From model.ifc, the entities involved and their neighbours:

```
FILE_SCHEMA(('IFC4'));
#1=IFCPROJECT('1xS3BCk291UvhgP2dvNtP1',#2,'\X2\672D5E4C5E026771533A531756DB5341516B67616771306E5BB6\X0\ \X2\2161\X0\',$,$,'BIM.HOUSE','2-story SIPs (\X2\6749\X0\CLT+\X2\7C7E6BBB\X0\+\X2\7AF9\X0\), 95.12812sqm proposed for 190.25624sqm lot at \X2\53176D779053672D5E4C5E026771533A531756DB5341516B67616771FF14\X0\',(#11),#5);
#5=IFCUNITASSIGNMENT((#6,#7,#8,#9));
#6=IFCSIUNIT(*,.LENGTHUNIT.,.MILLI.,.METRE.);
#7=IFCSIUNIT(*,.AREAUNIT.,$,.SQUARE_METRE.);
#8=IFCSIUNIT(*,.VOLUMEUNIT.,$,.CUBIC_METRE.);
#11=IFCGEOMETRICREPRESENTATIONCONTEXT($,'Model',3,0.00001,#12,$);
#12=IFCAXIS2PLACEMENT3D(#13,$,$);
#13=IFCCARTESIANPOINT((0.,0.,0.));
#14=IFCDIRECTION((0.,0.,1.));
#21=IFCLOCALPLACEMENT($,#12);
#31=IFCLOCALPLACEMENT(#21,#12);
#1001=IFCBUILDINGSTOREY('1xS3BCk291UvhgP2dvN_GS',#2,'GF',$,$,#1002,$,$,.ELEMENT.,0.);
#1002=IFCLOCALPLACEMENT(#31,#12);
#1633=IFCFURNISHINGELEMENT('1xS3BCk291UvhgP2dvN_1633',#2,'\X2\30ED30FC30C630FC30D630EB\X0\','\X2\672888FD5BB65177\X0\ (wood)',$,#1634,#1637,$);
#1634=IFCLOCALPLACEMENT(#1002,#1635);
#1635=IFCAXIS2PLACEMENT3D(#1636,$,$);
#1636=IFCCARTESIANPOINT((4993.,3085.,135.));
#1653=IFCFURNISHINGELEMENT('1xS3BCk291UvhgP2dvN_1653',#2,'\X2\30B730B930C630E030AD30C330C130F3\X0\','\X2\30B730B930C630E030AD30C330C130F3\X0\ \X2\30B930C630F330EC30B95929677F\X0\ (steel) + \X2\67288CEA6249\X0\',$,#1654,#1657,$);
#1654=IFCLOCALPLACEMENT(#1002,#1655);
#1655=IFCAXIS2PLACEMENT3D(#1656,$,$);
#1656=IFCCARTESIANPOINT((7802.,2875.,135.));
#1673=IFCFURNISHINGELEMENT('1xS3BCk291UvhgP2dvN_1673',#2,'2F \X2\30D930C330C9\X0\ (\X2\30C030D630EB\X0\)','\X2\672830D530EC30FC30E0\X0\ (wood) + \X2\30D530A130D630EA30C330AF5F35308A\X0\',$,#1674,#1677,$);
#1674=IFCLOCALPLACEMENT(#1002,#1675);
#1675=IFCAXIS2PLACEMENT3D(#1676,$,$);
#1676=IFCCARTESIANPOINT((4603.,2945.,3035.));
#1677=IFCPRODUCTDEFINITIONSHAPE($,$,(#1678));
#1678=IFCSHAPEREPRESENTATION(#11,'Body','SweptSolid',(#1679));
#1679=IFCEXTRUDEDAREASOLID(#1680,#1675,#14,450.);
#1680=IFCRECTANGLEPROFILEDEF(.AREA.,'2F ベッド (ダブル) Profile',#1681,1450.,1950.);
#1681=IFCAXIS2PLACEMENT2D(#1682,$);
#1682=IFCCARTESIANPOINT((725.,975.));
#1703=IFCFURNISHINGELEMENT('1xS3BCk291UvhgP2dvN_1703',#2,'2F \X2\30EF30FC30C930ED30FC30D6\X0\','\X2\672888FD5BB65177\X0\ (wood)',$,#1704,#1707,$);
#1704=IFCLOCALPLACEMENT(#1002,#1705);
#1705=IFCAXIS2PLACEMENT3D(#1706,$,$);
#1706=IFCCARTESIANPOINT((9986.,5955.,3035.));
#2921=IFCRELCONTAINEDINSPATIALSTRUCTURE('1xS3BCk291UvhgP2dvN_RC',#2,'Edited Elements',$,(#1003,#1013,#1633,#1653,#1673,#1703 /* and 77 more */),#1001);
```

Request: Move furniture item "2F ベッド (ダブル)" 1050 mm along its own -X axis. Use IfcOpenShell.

```python
import ifcopenshell
import ifcopenshell.api.geometry
import ifcopenshell.util.placement
import ifcopenshell.util.unit

model = ifcopenshell.open("model.ifc")
unit_scale = ifcopenshell.util.unit.calculate_unit_scale(model)

item = model.by_guid("1xS3BCk291UvhgP2dvN_1673")
matrix = ifcopenshell.util.placement.get_local_placement(item.ObjectPlacement)
matrix[:3, 3] -= matrix[:3, 0] * 1.05 / unit_scale
ifcopenshell.api.geometry.edit_object_placement(model, product=item, matrix=matrix, is_si=False)

print(ifcopenshell.util.placement.get_local_placement(item.ObjectPlacement).round(3) + 0.0)

model.write("model-out.ifc")
```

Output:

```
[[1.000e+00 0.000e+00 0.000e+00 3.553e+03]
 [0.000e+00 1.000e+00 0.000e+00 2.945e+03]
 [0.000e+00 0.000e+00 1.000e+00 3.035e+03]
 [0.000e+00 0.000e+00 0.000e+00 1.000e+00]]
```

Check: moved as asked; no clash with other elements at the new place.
